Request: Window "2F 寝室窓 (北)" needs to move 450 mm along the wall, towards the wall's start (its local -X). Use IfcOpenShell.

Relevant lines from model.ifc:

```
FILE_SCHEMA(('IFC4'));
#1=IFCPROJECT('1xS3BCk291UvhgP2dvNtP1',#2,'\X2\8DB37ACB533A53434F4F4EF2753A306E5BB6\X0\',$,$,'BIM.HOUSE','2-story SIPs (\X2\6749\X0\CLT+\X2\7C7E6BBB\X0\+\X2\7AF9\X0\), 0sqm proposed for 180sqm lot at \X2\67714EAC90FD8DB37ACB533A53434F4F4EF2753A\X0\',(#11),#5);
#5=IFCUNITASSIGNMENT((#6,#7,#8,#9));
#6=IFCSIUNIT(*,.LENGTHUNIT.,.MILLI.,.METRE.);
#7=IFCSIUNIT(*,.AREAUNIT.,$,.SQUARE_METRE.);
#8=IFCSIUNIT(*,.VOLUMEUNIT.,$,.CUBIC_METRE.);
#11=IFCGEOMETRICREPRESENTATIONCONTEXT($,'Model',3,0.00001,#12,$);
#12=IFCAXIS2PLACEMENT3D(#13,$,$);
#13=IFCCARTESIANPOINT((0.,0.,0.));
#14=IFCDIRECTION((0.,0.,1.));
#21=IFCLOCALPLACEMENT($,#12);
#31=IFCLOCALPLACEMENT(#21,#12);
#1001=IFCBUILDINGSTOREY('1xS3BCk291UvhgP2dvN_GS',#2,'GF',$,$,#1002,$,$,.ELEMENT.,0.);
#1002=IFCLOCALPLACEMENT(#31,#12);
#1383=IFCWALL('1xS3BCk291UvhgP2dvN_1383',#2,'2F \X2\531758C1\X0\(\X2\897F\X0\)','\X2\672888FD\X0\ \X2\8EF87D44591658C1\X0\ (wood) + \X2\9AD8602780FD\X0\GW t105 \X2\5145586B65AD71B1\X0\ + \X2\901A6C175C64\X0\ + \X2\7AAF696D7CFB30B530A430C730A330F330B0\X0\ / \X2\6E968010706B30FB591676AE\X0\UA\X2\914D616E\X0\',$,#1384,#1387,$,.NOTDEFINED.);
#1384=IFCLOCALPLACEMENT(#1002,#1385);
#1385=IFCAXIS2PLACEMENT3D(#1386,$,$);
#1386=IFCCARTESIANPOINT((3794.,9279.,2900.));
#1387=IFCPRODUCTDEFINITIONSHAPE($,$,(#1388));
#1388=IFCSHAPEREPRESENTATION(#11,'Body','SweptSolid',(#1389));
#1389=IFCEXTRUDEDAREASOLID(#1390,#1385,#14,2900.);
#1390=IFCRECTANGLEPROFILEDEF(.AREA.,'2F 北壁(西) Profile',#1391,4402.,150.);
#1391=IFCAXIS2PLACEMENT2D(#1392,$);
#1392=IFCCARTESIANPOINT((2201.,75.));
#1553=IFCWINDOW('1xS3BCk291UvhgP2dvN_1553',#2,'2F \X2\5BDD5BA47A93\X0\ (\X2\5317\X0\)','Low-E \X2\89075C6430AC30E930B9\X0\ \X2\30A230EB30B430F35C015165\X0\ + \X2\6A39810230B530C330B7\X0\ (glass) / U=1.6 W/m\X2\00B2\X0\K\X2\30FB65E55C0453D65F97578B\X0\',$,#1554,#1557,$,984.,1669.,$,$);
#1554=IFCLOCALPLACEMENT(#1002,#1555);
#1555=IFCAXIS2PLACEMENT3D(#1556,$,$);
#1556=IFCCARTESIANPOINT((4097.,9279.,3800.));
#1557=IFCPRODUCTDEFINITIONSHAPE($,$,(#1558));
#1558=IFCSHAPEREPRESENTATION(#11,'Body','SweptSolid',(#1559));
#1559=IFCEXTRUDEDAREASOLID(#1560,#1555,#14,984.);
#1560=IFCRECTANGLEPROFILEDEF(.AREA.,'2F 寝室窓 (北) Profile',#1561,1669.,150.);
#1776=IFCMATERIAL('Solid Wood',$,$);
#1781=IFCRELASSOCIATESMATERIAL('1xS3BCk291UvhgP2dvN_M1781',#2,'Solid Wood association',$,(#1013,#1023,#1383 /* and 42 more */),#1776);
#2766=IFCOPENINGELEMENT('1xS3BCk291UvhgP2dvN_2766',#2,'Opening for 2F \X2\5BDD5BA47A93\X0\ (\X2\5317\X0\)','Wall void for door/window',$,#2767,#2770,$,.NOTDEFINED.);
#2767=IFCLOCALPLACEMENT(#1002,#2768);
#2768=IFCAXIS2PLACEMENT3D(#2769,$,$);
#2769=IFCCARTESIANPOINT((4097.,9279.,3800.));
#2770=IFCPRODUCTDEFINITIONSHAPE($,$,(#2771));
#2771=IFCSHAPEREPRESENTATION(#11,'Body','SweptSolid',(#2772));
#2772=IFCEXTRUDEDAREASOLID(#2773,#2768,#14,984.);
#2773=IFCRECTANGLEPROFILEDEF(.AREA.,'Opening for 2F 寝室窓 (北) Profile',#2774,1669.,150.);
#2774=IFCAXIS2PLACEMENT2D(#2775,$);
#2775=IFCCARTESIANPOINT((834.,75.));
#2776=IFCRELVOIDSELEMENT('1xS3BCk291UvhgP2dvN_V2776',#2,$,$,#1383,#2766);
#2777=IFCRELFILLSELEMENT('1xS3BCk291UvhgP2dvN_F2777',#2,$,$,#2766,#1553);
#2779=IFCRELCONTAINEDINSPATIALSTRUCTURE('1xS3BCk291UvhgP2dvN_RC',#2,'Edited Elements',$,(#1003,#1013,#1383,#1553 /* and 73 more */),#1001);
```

```python
import ifcopenshell
import ifcopenshell.api.geometry
import ifcopenshell.util.placement
import ifcopenshell.util.unit

model = ifcopenshell.open("model.ifc")
unit_scale = ifcopenshell.util.unit.calculate_unit_scale(model)

window = model.by_guid("1xS3BCk291UvhgP2dvN_1553")
opening = window.FillsVoids[0].RelatingOpeningElement
wall = opening.VoidsElements[0].RelatingBuildingElement

wall_matrix = ifcopenshell.util.placement.get_local_placement(wall.ObjectPlacement)
shift = wall_matrix[:3, 0] * -0.45 / unit_scale
before = ifcopenshell.util.placement.get_local_placement(window.ObjectPlacement)[:3, 3].copy()

# The window is not placed relative to its opening, so move both.
for product in (opening, window):
    matrix = ifcopenshell.util.placement.get_local_placement(product.ObjectPlacement)
    matrix[:3, 3] += shift
    ifcopenshell.api.geometry.edit_object_placement(model, product=product, matrix=matrix, is_si=False)

after = ifcopenshell.util.placement.get_local_placement(window.ObjectPlacement)[:3, 3]
print("window moved by", (after - before).round(3) + 0.0)

model.write("model_edited.ifc")
```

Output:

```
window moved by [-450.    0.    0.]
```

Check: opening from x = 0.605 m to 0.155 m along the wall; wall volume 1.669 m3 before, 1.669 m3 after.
